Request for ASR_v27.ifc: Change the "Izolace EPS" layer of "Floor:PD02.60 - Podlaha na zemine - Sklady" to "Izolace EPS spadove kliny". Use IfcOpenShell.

First a look at what the model holds.

```python
import ifcopenshell
import ifcopenshell.util.element

model = ifcopenshell.open("ASR_v27.ifc")
print(model.schema)
for layer_set in model.by_type("IfcMaterialLayerSet"):
    if layer_set.LayerSetName == "Floor:PD02.60 - Podlaha na zemine - Sklady":
        for layer in layer_set.MaterialLayers:
            print(layer.id(), layer.Material and layer.Material.Name, layer.LayerThickness, sep=" | ")
        print(len(ifcopenshell.util.element.get_elements_by_material(model, layer_set)), "elements and types use it")
print(sorted(m.Name for m in model.by_type("IfcMaterial") if m.Name)[:60])
```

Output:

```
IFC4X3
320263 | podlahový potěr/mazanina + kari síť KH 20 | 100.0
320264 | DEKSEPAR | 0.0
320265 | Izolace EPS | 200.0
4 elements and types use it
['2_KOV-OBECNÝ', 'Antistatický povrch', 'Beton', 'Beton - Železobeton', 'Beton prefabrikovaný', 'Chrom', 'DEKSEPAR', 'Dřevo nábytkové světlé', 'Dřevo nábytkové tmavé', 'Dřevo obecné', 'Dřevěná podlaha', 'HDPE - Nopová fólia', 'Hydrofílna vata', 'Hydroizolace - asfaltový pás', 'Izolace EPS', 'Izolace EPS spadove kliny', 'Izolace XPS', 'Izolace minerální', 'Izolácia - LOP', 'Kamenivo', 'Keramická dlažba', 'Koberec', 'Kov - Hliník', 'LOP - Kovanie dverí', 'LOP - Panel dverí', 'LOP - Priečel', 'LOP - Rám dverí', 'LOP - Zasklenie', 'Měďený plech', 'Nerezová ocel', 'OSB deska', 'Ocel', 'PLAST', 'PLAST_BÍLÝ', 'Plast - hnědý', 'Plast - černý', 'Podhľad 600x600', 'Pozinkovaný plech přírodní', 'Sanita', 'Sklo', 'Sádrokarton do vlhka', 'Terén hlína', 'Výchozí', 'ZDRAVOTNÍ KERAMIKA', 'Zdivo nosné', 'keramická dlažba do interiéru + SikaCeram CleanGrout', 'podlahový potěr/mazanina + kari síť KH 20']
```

```python
import ifcopenshell
import ifcopenshell.api.material

model = ifcopenshell.open("ASR_v27.ifc")

layer_set = next(s for s in model.by_type("IfcMaterialLayerSet") if s.LayerSetName == "Floor:PD02.60 - Podlaha na zemine - Sklady")
layer = next(l for l in layer_set.MaterialLayers if l.Material and l.Material.Name == "Izolace EPS")
material = next(m for m in model.by_type("IfcMaterial") if m.Name == "Izolace EPS spadove kliny")

# Point this one layer at the other material; renaming the old one would change it everywhere.
ifcopenshell.api.material.edit_layer(model, layer=layer, attributes={"Name": material.Name}, material=material)

print([l.Material.Name if l.Material else None for l in layer_set.MaterialLayers])

model.write("ASR_v27_v2.ifc")
```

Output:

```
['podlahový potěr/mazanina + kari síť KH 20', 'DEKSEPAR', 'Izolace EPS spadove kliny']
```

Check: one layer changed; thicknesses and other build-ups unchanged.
